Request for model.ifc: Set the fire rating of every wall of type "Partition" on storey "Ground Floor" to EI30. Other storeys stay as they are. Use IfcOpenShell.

First a look at what the model holds.

```python
import ifcopenshell
import ifcopenshell.util.element

model = ifcopenshell.open("model.ifc")
print(model.schema)
storey = next(s for s in model.by_type("IfcBuildingStorey") if s.Name == "Ground Floor")
walls = [e for e in ifcopenshell.util.element.get_decomposition(storey) if e.is_a("IfcWall")]
seen = {}
for e in walls:
    element_type = ifcopenshell.util.element.get_type(e)
    key = (element_type.Name if element_type != e and element_type else None, ifcopenshell.util.element.get_pset(e, "Pset_WallCommon", "FireRating"))
    seen[key] = seen.get(key, 0) + 1
for (name, value), count in sorted(seen.items(), key=str):
    print(count, "x", name, "|", value)
```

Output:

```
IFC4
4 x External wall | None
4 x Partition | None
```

```python
import ifcopenshell
import ifcopenshell.api.pset
import ifcopenshell.util.element

model = ifcopenshell.open("model.ifc")

storey = next(s for s in model.by_type("IfcBuildingStorey") if s.Name == "Ground Floor")
walls = [e for e in ifcopenshell.util.element.get_decomposition(storey) if e.is_a("IfcWall")]

count = 0
for e in walls:
    element_type = ifcopenshell.util.element.get_type(e)
    if element_type in (None, e) or element_type.Name != "Partition":
        continue
    # add_pset returns the element's existing set when there is one.
    pset = ifcopenshell.api.pset.add_pset(model, product=e, name="Pset_WallCommon")
    ifcopenshell.api.pset.edit_pset(model, pset=pset, properties={"FireRating": "EI30"})
    count += 1

print(count, "walls updated")

model.write("model_v2.ifc")
```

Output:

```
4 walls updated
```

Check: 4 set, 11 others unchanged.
